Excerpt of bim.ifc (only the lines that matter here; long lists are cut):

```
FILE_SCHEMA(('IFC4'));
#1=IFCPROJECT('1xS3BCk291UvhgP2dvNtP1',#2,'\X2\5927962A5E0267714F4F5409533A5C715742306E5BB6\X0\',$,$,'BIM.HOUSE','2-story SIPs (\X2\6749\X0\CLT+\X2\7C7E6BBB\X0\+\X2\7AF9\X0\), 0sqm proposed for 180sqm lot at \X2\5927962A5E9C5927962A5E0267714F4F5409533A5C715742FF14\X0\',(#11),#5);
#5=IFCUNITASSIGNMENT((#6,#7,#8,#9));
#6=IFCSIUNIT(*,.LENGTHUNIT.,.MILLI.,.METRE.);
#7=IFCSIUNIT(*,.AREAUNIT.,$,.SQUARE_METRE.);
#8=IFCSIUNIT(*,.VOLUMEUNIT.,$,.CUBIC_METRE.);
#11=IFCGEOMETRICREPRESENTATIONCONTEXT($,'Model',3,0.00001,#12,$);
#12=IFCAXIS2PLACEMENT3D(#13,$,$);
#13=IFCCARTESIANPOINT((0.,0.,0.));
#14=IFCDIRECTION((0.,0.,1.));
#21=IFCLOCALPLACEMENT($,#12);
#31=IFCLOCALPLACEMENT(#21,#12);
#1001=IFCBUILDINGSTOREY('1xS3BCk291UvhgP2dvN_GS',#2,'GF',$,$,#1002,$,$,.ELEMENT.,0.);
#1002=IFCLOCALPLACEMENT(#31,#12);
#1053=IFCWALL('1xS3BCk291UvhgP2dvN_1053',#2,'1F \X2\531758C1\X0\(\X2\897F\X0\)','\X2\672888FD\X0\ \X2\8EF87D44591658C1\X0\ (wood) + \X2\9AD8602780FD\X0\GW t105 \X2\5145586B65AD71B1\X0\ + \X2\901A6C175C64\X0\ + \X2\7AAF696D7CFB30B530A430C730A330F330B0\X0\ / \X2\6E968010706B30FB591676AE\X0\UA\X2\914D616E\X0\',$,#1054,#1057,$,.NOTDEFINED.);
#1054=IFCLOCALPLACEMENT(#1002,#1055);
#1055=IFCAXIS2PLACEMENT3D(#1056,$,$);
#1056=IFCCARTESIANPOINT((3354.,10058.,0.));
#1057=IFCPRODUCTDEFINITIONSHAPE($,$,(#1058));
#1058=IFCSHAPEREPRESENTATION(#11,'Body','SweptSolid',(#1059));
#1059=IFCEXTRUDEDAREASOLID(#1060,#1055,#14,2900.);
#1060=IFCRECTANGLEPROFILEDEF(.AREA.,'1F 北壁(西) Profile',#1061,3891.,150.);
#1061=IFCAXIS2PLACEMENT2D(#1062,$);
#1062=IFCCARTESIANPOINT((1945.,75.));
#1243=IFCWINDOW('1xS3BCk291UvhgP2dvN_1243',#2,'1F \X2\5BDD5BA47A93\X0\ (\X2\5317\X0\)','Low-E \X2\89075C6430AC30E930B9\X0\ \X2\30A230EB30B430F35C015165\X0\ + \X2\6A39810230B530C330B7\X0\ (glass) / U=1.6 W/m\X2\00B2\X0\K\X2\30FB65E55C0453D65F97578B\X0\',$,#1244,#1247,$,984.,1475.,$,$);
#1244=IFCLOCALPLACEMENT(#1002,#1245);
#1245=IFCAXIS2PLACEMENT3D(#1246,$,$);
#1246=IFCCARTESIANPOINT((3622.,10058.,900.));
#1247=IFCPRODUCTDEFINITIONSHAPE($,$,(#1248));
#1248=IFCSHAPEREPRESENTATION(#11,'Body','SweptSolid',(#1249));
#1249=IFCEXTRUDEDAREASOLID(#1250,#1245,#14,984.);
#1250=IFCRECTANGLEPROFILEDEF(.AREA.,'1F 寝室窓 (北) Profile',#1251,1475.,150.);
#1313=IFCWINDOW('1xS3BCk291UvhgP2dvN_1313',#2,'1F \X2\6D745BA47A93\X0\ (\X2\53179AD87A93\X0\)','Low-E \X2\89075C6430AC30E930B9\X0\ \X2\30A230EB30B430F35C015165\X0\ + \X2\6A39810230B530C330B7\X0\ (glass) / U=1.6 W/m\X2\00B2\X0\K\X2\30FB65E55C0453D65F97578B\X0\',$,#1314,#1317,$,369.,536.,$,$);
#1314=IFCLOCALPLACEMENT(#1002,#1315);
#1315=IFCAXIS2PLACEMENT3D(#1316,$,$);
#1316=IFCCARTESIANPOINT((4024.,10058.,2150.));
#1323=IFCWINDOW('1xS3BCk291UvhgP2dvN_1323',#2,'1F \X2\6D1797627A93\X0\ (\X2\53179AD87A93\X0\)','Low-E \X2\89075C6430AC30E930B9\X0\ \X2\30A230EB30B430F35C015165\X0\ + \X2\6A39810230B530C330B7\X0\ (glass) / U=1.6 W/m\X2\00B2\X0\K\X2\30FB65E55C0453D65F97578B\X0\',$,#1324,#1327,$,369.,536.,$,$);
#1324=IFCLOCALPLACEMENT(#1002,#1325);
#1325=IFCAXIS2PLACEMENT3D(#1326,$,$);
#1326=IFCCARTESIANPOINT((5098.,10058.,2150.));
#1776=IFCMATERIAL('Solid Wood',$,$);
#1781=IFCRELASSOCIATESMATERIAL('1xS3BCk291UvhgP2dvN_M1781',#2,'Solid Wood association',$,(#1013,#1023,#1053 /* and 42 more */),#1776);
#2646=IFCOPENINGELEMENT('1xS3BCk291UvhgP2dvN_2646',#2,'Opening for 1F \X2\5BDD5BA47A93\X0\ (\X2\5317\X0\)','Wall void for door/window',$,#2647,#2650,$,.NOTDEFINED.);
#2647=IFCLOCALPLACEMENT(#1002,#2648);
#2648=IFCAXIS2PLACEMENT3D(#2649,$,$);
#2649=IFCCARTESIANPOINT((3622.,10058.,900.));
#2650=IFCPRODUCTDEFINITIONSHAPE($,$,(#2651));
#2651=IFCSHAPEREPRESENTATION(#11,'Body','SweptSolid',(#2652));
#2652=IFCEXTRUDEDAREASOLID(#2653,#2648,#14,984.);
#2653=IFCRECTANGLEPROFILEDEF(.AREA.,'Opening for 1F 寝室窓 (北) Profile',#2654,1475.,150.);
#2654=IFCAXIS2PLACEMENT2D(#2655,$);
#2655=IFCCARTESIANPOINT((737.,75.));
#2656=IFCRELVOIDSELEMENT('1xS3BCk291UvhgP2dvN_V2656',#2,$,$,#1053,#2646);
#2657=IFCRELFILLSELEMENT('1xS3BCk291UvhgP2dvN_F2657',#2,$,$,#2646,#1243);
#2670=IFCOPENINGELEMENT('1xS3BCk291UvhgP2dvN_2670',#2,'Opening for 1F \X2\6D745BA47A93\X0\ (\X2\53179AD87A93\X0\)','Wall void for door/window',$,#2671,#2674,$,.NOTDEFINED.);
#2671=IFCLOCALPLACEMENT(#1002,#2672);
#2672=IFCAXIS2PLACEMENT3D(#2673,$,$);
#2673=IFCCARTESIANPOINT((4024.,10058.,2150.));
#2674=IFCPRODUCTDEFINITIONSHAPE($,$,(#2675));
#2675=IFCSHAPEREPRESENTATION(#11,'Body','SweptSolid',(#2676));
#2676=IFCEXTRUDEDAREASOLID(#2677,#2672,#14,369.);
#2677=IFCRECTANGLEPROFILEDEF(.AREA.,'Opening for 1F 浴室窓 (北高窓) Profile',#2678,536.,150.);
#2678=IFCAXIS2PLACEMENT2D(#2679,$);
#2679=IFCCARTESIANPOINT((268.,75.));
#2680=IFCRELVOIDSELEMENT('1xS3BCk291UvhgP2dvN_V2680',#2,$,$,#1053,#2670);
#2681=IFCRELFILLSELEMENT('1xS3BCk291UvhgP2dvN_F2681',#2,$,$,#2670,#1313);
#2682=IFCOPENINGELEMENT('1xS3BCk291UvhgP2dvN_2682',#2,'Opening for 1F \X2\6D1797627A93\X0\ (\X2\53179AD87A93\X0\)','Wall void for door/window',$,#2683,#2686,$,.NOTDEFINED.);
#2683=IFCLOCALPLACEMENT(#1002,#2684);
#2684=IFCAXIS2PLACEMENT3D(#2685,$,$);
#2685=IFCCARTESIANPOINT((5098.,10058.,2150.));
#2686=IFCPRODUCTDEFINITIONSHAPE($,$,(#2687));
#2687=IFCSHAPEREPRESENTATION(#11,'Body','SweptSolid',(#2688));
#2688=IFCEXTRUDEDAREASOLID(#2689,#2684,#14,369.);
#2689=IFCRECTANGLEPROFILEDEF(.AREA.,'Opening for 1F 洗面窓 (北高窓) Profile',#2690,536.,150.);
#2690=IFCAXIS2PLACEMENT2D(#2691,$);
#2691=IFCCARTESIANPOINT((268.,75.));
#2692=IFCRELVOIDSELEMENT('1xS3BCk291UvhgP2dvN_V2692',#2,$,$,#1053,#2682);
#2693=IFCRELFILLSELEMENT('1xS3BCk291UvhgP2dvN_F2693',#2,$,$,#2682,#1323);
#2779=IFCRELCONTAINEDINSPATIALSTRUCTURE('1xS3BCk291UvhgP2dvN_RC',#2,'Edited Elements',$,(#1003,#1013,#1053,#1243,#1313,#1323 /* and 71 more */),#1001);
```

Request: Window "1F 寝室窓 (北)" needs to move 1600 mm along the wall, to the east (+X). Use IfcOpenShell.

```python
import ifcopenshell
import ifcopenshell.api.geometry
import ifcopenshell.util.placement
import ifcopenshell.util.unit

model = ifcopenshell.open("bim.ifc")
unit_scale = ifcopenshell.util.unit.calculate_unit_scale(model)

window = model.by_id(1243)
opening = window.FillsVoids[0].RelatingOpeningElement
wall = opening.VoidsElements[0].RelatingBuildingElement

wall_matrix = ifcopenshell.util.placement.get_local_placement(wall.ObjectPlacement)
shift = wall_matrix[:3, 0] * 1.6 / unit_scale
before = ifcopenshell.util.placement.get_local_placement(window.ObjectPlacement)[:3, 3].copy()

# The window is not placed relative to its opening, so move both.
for product in (opening, window):
    matrix = ifcopenshell.util.placement.get_local_placement(product.ObjectPlacement)
    matrix[:3, 3] += shift
    ifcopenshell.api.geometry.edit_object_placement(model, product=product, matrix=matrix, is_si=False)

after = ifcopenshell.util.placement.get_local_placement(window.ObjectPlacement)[:3, 3]
print("window moved by", (after - before).round(3) + 0.0)

model.write("bim_rev.ifc")
```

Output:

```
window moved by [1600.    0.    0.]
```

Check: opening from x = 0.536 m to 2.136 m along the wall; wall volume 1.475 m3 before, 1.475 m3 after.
